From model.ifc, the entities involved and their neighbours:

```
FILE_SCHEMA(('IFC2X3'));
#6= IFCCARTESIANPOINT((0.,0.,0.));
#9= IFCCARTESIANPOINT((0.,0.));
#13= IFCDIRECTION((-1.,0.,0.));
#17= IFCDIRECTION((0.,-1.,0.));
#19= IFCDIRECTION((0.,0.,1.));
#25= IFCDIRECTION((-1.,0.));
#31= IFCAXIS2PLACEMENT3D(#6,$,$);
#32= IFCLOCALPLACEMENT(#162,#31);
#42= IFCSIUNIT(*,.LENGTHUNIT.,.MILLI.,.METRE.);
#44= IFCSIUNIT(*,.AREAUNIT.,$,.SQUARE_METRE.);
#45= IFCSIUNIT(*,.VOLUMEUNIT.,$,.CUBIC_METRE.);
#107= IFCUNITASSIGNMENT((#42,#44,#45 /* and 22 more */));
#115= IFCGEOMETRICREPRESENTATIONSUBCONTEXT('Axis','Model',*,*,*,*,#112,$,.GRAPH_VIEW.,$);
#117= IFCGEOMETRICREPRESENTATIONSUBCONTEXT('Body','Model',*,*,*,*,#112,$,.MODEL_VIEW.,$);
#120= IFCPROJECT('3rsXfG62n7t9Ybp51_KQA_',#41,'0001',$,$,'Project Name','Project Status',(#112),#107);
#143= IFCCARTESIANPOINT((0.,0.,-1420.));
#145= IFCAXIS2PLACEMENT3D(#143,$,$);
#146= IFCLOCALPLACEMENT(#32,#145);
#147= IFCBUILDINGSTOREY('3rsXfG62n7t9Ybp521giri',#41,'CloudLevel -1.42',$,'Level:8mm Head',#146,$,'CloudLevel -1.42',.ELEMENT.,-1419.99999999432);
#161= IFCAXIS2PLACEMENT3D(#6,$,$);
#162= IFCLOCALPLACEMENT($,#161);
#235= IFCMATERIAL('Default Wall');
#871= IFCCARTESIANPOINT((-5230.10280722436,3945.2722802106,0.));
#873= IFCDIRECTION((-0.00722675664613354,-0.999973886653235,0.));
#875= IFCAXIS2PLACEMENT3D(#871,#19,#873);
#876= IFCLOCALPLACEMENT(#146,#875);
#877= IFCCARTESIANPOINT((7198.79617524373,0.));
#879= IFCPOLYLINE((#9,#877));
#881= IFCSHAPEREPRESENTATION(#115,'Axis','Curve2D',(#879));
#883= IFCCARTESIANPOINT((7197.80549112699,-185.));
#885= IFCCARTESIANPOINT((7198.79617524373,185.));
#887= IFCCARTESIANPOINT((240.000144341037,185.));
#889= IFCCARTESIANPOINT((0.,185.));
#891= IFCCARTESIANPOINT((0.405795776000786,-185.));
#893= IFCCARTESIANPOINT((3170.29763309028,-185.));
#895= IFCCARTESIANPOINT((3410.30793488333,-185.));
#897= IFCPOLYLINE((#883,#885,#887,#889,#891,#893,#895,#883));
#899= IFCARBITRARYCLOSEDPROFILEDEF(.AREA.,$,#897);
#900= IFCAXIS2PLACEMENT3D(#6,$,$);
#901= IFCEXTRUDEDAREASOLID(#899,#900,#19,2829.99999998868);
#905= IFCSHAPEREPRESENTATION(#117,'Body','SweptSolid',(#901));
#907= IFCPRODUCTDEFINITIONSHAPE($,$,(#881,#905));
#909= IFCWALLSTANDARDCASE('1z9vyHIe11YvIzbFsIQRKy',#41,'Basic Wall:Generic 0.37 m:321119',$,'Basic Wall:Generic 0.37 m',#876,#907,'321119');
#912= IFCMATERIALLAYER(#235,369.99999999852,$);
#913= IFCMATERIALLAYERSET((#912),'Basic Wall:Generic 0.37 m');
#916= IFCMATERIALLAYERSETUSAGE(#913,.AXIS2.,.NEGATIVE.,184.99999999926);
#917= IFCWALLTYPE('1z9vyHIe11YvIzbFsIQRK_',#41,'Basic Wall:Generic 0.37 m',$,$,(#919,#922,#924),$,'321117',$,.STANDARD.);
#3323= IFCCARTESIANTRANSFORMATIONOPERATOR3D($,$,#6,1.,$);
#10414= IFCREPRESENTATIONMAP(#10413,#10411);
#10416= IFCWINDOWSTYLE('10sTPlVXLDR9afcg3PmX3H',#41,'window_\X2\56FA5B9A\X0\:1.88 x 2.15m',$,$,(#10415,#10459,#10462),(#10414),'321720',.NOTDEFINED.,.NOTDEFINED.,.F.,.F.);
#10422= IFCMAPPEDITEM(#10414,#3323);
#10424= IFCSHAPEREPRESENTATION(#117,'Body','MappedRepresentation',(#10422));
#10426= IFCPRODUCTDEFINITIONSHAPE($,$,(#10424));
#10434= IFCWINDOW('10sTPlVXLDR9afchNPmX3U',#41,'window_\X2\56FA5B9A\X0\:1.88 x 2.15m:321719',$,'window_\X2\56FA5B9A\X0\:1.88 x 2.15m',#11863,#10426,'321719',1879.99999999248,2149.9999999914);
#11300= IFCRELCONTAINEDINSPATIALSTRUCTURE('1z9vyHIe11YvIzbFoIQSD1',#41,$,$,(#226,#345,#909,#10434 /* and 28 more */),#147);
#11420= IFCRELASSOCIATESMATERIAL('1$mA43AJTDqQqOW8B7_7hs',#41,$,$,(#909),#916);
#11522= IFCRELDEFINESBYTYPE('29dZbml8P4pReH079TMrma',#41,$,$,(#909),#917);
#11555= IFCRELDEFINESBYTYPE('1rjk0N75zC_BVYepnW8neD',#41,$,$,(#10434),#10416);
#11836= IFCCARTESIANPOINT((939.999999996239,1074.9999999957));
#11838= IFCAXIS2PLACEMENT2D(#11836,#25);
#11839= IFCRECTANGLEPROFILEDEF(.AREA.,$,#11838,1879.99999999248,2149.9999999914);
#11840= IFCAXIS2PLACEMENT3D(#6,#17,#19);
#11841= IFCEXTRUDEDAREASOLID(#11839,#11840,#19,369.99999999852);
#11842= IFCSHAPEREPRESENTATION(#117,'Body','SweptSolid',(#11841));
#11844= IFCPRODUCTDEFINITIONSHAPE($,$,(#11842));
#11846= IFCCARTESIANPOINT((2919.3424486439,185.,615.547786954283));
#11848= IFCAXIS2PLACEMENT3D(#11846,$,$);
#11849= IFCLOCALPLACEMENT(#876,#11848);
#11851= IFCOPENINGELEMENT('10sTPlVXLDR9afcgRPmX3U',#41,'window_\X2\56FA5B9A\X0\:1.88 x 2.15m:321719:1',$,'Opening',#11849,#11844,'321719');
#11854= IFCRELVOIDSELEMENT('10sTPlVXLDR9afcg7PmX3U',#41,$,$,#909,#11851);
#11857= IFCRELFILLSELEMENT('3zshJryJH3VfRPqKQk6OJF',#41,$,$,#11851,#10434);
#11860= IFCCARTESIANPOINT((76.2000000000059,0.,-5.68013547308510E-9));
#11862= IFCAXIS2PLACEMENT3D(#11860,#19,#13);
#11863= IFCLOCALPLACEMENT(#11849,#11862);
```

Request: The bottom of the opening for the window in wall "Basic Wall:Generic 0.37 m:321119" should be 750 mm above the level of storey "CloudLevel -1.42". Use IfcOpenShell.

```python
import numpy as np
import ifcopenshell
import ifcopenshell.api.geometry
import ifcopenshell.geom
import ifcopenshell.util.element
import ifcopenshell.util.placement
import ifcopenshell.util.shape
import ifcopenshell.util.unit

model = ifcopenshell.open("model.ifc")
unit_scale = ifcopenshell.util.unit.calculate_unit_scale(model)

window = model.by_guid("10sTPlVXLDR9afchNPmX3U")
opening = window.FillsVoids[0].RelatingOpeningElement
storey = ifcopenshell.util.element.get_container(window, ifc_class="IfcBuildingStorey")
level = ifcopenshell.util.placement.get_local_placement(storey.ObjectPlacement)[2, 3]

# The opening's origin need not be at the sill, so measure its lowest point.
shape = ifcopenshell.geom.create_shape(ifcopenshell.geom.settings(), opening)
bottom = ifcopenshell.util.shape.get_shape_bottom_elevation(shape, shape.geometry) / unit_scale
dz = level + 0.75 / unit_scale - bottom

shift = np.array([0.0, 0.0, dz])
# The window is placed relative to its opening, so it follows when the opening moves.
matrix = ifcopenshell.util.placement.get_local_placement(opening.ObjectPlacement)
matrix[:3, 3] += shift
ifcopenshell.api.geometry.edit_object_placement(
    model, product=opening, matrix=matrix, is_si=False, should_transform_children=True
)

print(f"moved by {dz * unit_scale:+.3f} m")

model.write("model_updated.ifc")
```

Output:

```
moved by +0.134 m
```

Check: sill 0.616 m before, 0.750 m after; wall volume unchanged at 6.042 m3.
